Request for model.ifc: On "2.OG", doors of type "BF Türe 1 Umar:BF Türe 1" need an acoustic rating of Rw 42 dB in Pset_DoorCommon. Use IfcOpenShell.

First a look at what the model holds.

```python
import ifcopenshell
import ifcopenshell.util.element

model = ifcopenshell.open("model.ifc")
print(model.schema)
storey = next(s for s in model.by_type("IfcBuildingStorey") if s.Name == "2.OG")
doors = [e for e in ifcopenshell.util.element.get_decomposition(storey) if e.is_a("IfcDoor")]
seen = {}
for e in doors:
    element_type = ifcopenshell.util.element.get_type(e)
    key = (element_type.Name if element_type != e and element_type else None, ifcopenshell.util.element.get_pset(e, "Pset_DoorCommon", "AcousticRating"))
    seen[key] = seen.get(key, 0) + 1
for (name, value), count in sorted(seen.items(), key=str):
    print(count, "x", name, "|", value)
```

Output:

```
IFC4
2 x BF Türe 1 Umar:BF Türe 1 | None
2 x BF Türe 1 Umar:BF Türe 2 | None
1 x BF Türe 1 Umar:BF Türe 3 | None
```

```python
import ifcopenshell
import ifcopenshell.api.pset
import ifcopenshell.util.element

model = ifcopenshell.open("model.ifc")

storey = next(s for s in model.by_type("IfcBuildingStorey") if s.Name == "2.OG")
doors = [e for e in ifcopenshell.util.element.get_decomposition(storey) if e.is_a("IfcDoor")]

count = 0
for e in doors:
    element_type = ifcopenshell.util.element.get_type(e)
    if element_type in (None, e) or element_type.Name != "BF Türe 1 Umar:BF Türe 1":
        continue
    # add_pset returns the element's existing set when there is one.
    pset = ifcopenshell.api.pset.add_pset(model, product=e, name="Pset_DoorCommon")
    ifcopenshell.api.pset.edit_pset(model, pset=pset, properties={"AcousticRating": "Rw 42 dB"})
    count += 1

print(count, "doors updated")

model.write("model-out.ifc")
```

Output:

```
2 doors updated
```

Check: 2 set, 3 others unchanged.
